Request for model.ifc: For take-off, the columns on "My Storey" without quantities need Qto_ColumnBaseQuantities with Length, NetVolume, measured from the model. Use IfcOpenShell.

First a look at what the model holds.

```python
import ifcopenshell
import ifcopenshell.util.element
import ifcopenshell.util.unit

model = ifcopenshell.open("model.ifc")
print(model.schema)
for unit_type in ("LENGTHUNIT", "AREAUNIT", "VOLUMEUNIT"):
    print(unit_type, ifcopenshell.util.unit.calculate_unit_scale(model, unit_type))
storey = next(s for s in model.by_type("IfcBuildingStorey") if s.Name == "My Storey")
columns = [e for e in ifcopenshell.util.element.get_decomposition(storey) if e.is_a("IfcColumn")]
for e in sorted(columns, key=lambda e: e.id()):
    print(e.id(), e.is_a(), e.Name, list(ifcopenshell.util.element.get_psets(e, qtos_only=True)), sep=" | ")
```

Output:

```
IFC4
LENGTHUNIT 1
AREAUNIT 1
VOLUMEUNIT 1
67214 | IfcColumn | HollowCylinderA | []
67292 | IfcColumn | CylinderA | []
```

```python
import ifcopenshell
import ifcopenshell.api.pset
import ifcopenshell.geom
import ifcopenshell.util.element
import ifcopenshell.util.shape
import ifcopenshell.util.unit

model = ifcopenshell.open("model.ifc")
unit_scale = ifcopenshell.util.unit.calculate_unit_scale(model)
volume_scale = ifcopenshell.util.unit.calculate_unit_scale(model, "VOLUMEUNIT")
settings = ifcopenshell.geom.settings()

storey = next(s for s in model.by_type("IfcBuildingStorey") if s.Name == "My Storey")
columns = [e for e in ifcopenshell.util.element.get_decomposition(storey) if e.is_a("IfcColumn")]

for e in sorted(columns, key=lambda e: e.id()):
    if ifcopenshell.util.element.get_psets(e, qtos_only=True, should_inherit=False):
        continue
    # Geometry comes back in metres, in the element's own axes.
    shape = ifcopenshell.geom.create_shape(settings, e)
    values = {
        "Length": ifcopenshell.util.shape.get_z(shape.geometry) / unit_scale,
        "NetVolume": ifcopenshell.util.shape.get_volume(shape.geometry) / volume_scale,
    }
    qto = ifcopenshell.api.pset.add_qto(model, product=e, name="Qto_ColumnBaseQuantities")
    ifcopenshell.api.pset.edit_qto(model, qto=qto, properties=values)
    print(e.id(), {k: round(v, 3) for k, v in values.items()})

model.write("model_v2.ifc")
```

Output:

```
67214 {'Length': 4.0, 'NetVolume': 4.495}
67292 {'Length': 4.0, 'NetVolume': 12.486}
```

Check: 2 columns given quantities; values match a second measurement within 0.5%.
